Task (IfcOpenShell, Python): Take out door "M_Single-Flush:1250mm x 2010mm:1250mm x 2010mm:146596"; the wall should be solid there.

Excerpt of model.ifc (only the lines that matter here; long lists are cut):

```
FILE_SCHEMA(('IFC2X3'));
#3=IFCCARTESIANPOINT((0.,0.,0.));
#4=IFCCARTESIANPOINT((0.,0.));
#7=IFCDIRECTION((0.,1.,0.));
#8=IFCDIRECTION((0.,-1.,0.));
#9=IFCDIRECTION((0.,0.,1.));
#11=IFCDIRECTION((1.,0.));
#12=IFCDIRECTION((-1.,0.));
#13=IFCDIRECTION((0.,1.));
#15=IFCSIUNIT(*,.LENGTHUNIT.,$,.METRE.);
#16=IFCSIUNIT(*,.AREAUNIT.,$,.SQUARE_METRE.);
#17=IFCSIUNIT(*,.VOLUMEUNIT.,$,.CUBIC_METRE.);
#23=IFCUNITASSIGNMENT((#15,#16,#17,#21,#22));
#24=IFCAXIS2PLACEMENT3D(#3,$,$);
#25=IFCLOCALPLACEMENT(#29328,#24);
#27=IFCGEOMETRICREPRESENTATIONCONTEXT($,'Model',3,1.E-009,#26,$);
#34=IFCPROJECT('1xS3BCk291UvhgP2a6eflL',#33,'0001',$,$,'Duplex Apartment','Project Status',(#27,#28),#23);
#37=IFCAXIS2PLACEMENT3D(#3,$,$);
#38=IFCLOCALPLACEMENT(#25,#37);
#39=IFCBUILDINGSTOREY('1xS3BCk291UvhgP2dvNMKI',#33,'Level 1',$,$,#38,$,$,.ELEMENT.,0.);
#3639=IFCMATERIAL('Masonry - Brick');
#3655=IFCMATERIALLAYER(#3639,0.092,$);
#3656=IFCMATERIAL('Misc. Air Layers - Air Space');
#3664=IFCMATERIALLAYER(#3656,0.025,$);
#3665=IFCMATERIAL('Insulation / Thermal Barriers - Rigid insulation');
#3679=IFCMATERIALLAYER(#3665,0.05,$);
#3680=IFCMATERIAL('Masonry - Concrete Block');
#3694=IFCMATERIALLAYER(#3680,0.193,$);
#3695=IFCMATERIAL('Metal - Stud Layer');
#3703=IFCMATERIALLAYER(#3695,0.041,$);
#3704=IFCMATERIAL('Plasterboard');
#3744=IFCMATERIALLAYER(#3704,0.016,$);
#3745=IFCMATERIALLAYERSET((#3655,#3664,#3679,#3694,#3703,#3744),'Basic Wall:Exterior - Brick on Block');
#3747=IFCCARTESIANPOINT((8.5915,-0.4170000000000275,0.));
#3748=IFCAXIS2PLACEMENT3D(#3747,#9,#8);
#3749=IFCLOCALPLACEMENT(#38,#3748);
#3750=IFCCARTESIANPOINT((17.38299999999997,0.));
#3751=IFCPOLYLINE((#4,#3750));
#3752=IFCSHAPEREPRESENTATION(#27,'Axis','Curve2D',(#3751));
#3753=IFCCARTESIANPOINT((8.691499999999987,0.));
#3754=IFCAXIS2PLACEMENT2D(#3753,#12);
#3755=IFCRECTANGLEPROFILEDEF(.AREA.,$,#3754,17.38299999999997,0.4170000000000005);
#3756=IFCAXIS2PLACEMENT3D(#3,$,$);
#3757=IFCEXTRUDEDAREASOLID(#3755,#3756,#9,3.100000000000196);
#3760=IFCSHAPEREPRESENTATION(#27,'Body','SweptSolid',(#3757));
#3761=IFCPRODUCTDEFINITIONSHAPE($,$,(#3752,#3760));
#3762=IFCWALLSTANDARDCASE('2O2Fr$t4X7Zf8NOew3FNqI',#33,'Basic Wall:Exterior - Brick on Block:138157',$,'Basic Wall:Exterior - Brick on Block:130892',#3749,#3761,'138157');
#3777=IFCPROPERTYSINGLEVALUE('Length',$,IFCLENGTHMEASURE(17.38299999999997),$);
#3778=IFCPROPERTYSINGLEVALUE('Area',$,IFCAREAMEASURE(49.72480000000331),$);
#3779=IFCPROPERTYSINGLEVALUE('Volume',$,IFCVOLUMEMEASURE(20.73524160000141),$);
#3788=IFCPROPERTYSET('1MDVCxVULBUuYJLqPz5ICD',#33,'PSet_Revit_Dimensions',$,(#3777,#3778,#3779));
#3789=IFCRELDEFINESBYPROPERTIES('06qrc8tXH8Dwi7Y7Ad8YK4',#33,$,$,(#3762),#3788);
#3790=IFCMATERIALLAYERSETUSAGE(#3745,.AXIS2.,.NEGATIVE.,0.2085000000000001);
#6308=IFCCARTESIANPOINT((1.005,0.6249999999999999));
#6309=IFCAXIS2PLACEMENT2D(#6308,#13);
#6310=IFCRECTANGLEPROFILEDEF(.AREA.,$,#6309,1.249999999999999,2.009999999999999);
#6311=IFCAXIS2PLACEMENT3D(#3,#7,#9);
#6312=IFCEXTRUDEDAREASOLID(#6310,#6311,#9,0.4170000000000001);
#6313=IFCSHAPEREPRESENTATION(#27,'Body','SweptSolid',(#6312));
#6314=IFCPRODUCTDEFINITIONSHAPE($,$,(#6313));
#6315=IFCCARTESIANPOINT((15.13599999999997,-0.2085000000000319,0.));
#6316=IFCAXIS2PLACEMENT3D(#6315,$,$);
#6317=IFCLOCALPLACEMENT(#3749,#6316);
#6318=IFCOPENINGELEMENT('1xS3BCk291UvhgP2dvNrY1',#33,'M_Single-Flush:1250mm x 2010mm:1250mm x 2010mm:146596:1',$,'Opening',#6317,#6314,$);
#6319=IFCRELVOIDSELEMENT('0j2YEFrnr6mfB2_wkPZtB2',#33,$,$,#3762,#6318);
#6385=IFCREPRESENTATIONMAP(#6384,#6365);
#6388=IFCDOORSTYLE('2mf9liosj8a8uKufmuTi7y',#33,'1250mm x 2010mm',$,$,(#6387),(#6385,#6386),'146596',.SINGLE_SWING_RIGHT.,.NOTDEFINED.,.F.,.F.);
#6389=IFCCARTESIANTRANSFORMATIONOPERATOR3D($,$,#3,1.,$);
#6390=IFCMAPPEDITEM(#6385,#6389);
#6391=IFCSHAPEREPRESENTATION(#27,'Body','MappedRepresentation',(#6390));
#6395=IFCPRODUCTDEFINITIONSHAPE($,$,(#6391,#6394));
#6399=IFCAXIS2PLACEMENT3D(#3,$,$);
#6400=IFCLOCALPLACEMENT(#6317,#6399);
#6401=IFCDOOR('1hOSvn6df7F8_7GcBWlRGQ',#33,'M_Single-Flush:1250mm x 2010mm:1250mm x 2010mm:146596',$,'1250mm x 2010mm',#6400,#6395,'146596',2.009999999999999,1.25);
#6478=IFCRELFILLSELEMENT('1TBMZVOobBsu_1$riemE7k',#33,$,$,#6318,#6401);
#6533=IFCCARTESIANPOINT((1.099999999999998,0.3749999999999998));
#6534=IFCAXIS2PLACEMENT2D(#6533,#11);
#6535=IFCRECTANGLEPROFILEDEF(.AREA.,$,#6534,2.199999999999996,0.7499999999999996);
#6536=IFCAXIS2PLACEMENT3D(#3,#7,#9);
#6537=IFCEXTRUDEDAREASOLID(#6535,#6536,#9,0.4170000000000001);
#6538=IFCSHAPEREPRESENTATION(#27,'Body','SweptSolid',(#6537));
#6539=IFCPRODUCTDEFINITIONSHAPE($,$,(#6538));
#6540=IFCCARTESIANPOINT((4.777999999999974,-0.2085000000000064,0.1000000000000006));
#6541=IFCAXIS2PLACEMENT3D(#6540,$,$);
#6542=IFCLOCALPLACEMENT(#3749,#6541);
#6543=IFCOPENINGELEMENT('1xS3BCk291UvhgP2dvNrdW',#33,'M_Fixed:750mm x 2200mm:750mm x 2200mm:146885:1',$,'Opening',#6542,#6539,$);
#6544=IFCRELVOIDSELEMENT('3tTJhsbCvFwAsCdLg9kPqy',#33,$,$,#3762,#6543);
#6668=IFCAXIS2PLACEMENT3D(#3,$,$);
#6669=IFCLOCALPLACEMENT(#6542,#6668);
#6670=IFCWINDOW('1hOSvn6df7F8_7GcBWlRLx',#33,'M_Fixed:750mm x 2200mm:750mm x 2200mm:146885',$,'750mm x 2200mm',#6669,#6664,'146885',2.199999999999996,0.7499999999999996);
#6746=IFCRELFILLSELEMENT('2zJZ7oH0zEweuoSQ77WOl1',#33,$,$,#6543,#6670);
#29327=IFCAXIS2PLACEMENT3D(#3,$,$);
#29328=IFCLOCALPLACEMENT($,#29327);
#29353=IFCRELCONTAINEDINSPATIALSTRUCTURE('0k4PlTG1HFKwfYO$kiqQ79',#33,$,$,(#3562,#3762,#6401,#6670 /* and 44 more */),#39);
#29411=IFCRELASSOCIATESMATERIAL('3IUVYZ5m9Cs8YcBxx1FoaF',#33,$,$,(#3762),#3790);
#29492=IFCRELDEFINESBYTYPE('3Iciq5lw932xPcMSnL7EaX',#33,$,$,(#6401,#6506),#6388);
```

```python
import ifcopenshell
import ifcopenshell.api.feature
import ifcopenshell.api.pset
import ifcopenshell.api.root
import ifcopenshell.geom
import ifcopenshell.util.element
import ifcopenshell.util.shape
import ifcopenshell.util.unit

model = ifcopenshell.open("model.ifc")
area_scale = ifcopenshell.util.unit.calculate_unit_scale(model, "AREAUNIT")
volume_scale = ifcopenshell.util.unit.calculate_unit_scale(model, "VOLUMEUNIT")
settings = ifcopenshell.geom.settings()


def volume(element):
    """Net volume in cubic metres, openings subtracted."""
    shape = ifcopenshell.geom.create_shape(settings, element)
    return ifcopenshell.util.shape.get_volume(shape.geometry)


door = model.by_guid("1hOSvn6df7F8_7GcBWlRGQ")
opening = door.FillsVoids[0].RelatingOpeningElement
wall = opening.VoidsElements[0].RelatingBuildingElement
before = volume(wall)

ifcopenshell.api.root.remove_product(model, product=door)
ifcopenshell.api.feature.remove_feature(model, feature=opening)

after = volume(wall)
thickness = 0.417  # wall thickness in metres

# Update the wall's stored quantities.
pset = model.by_id(ifcopenshell.util.element.get_pset(wall, "PSet_Revit_Dimensions", should_inherit=False)["id"])
ifcopenshell.api.pset.edit_pset(model, pset=pset, properties={
    "Area": model.create_entity("IfcAreaMeasure", after / thickness / area_scale),
    "Volume": model.create_entity("IfcVolumeMeasure", after / volume_scale),
})

print(f"wall volume {before:.3f} -> {after:.3f} m3")

model.write("model_edited.ifc")
```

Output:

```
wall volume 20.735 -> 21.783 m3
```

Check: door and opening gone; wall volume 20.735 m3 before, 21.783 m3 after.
